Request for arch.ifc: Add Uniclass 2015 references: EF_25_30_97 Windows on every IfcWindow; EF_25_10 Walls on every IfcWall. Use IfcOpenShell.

First a look at what the model holds.

```python
import ifcopenshell

model = ifcopenshell.open("arch.ifc")
print(model.schema)
print("classifications:", [c.Name for c in model.by_type("IfcClassification")])
for ifc_class in ("IfcDoor", "IfcRoof", "IfcStair", "IfcWall", "IfcWindow"):
    print(ifc_class, len(model.by_type(ifc_class)))
```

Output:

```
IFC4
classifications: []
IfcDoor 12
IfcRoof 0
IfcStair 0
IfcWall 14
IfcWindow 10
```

```python
import ifcopenshell
import ifcopenshell.api.classification

model = ifcopenshell.open("arch.ifc")

system = ifcopenshell.api.classification.add_classification(model, classification="Uniclass 2015")

codes = {
    "IfcWindow": ("EF_25_30_97", "Windows"),
    "IfcWall": ("EF_25_10", "Walls"),
}
for ifc_class, (code, name) in codes.items():
    products = model.by_type(ifc_class)
    ifcopenshell.api.classification.add_reference(
        model, products=products, classification=system, identification=code, name=name
    )
    print(code, len(products))

model.write("arch_edited.ifc")
```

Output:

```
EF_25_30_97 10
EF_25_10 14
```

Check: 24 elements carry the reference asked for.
